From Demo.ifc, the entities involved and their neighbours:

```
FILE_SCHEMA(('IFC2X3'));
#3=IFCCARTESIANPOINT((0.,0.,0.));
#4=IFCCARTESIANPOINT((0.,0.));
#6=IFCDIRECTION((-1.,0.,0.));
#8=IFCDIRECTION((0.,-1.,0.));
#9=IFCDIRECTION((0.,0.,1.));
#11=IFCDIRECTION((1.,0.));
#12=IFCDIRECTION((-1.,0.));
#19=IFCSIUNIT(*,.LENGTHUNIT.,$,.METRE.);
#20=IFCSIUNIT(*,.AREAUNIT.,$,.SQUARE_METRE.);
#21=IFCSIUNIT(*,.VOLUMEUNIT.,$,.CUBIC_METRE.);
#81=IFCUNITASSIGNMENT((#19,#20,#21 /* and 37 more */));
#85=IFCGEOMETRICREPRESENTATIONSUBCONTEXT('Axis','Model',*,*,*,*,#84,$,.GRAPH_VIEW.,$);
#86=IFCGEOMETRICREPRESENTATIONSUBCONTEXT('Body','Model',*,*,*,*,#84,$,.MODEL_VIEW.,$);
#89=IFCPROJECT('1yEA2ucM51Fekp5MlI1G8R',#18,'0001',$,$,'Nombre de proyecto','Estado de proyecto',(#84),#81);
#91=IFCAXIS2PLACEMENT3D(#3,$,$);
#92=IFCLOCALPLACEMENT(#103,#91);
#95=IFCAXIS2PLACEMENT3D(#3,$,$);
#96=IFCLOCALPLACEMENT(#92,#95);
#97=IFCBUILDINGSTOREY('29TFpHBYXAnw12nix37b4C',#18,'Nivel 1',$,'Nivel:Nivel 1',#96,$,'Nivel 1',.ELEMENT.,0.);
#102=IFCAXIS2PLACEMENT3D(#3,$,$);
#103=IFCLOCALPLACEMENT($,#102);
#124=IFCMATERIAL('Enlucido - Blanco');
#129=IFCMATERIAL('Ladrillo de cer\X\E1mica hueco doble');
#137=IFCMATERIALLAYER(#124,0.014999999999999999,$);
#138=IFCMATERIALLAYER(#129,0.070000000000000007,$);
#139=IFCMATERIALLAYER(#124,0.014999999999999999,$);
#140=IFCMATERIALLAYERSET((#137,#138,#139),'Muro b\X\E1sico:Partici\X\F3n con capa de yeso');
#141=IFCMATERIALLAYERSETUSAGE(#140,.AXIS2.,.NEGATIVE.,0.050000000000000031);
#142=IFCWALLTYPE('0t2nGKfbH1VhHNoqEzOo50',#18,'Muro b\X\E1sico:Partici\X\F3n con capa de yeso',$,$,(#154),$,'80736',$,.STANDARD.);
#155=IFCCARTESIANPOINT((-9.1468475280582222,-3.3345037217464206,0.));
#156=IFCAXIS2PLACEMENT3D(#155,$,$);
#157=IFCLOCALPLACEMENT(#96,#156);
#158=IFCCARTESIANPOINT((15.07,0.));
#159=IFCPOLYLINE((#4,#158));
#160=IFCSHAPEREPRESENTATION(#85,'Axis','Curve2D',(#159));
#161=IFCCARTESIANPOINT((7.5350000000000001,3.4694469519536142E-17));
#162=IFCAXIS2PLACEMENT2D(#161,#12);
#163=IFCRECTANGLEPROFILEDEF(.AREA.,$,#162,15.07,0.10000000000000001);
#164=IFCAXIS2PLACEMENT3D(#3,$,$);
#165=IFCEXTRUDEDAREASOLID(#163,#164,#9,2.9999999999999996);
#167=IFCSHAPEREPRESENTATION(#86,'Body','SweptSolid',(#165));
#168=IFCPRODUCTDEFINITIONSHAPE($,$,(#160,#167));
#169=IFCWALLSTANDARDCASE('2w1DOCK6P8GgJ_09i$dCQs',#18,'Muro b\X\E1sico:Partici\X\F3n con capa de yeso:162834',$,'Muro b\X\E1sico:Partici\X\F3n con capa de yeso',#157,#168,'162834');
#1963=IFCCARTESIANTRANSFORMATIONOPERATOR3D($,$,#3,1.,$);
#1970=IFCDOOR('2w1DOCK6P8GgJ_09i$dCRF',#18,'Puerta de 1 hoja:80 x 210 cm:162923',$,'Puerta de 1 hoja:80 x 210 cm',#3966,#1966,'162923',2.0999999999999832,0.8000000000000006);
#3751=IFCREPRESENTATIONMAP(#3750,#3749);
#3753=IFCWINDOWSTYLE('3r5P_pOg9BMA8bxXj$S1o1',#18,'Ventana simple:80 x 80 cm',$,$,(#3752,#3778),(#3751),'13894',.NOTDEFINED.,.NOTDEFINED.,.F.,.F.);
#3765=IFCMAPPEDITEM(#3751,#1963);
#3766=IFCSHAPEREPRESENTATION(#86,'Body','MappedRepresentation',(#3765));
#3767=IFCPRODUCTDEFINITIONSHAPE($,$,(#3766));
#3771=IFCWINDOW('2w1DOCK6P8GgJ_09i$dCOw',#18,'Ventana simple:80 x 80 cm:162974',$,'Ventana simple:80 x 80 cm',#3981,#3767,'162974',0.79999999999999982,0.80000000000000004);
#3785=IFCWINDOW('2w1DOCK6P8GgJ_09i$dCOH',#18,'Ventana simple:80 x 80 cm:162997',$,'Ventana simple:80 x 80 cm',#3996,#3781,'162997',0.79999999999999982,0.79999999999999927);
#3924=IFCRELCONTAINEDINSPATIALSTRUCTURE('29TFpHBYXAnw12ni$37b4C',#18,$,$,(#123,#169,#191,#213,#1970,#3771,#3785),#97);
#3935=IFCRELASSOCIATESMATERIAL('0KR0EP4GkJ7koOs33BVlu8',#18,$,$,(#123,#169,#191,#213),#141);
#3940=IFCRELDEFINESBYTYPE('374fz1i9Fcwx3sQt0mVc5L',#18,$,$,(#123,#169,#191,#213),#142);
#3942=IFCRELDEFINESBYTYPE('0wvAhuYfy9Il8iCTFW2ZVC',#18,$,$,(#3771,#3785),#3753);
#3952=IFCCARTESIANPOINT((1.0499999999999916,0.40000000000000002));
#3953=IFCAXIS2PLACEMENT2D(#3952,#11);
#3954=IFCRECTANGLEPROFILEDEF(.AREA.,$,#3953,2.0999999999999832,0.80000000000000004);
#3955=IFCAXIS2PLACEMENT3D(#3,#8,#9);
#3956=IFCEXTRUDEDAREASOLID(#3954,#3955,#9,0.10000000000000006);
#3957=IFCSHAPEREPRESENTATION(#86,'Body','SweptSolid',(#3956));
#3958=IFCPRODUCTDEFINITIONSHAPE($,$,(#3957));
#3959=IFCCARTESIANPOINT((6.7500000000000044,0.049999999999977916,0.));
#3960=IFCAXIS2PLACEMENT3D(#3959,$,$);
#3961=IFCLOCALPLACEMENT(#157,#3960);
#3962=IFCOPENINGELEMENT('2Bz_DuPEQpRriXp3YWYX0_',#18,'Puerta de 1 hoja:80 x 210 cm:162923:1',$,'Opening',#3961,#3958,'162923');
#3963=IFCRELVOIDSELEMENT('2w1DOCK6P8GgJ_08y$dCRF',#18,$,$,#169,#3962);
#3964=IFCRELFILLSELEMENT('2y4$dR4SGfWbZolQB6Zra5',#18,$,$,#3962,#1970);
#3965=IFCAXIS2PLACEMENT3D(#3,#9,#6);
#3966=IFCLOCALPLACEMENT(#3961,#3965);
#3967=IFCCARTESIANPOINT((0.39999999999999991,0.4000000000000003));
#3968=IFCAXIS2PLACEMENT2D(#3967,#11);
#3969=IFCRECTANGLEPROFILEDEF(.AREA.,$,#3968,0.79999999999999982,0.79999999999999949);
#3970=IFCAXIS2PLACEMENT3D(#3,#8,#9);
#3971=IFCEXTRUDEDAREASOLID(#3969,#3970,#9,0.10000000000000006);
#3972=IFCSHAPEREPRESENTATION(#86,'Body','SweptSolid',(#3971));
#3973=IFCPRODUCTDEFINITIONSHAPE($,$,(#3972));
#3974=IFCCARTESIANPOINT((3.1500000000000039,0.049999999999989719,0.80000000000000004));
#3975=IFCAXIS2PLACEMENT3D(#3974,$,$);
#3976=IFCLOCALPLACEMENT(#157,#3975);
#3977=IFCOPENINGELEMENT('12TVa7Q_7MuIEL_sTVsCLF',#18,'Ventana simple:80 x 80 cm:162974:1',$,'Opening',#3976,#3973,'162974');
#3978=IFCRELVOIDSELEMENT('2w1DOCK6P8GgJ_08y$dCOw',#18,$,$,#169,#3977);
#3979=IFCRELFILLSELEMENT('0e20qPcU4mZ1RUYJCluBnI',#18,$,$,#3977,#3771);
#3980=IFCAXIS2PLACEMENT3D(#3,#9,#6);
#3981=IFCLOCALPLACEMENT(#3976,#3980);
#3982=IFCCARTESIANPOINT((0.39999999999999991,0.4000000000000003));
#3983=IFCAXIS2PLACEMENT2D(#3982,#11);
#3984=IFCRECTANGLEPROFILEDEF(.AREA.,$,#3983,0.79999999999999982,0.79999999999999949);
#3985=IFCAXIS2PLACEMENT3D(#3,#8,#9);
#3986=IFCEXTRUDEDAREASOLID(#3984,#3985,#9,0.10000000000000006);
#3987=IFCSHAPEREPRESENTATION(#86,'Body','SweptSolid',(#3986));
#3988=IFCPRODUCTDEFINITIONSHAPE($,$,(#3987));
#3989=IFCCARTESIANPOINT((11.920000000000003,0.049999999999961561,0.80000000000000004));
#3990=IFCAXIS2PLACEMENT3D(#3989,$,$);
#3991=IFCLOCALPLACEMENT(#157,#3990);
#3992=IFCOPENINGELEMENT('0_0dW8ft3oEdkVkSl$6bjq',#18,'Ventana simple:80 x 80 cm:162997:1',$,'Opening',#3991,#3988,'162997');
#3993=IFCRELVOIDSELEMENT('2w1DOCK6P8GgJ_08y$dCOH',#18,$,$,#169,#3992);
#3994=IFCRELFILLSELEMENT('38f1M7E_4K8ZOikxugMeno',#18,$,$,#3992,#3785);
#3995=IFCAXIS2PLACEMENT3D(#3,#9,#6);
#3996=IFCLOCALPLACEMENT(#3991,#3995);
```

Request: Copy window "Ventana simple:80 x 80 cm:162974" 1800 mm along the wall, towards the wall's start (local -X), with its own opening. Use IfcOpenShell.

```python
import ifcopenshell
import ifcopenshell.api.feature
import ifcopenshell.api.geometry
import ifcopenshell.api.root
import ifcopenshell.geom
import ifcopenshell.util.element
import ifcopenshell.util.placement
import ifcopenshell.util.shape
import ifcopenshell.util.unit

model = ifcopenshell.open("Demo.ifc")
unit_scale = ifcopenshell.util.unit.calculate_unit_scale(model)
settings = ifcopenshell.geom.settings()


def volume(element):
    """Net volume in cubic metres, openings subtracted."""
    shape = ifcopenshell.geom.create_shape(settings, element)
    return ifcopenshell.util.shape.get_volume(shape.geometry)


def reuse_history(source, copy):
    """copy_class also copies each property set's owner history, people and application; keep the originals."""
    for rel in copy.IsDefinedBy:
        if rel.is_a("IfcRelDefinesByProperties") and (history := rel.RelatingPropertyDefinition.OwnerHistory):
            rel.RelatingPropertyDefinition.OwnerHistory = source.OwnerHistory
            ifcopenshell.util.element.remove_deep2(model, history)


window = model.by_id(3771)
opening = window.FillsVoids[0].RelatingOpeningElement
wall = opening.VoidsElements[0].RelatingBuildingElement
before = volume(wall)
shift = ifcopenshell.util.placement.get_local_placement(wall.ObjectPlacement)[:3, 0] * -1.8 / unit_scale

# copy_class copies the void relationship, type, container and properties, but no geometry.
new_opening = ifcopenshell.api.root.copy_class(model, product=opening)
new_opening.Representation = ifcopenshell.util.element.copy_deep(
    model, opening.Representation, exclude=["IfcGeometricRepresentationContext", "IfcRepresentationMap"]
)
new_opening.Name = "Ventana simple:80 x 80 cm"
new_opening.Tag = None
new_window = ifcopenshell.api.root.copy_class(model, product=window)
new_window.Representation = ifcopenshell.util.element.copy_deep(
    model, window.Representation, exclude=["IfcGeometricRepresentationContext", "IfcRepresentationMap"]
)
new_window.Name = "Ventana simple:80 x 80 cm"
new_window.Tag = None
reuse_history(window, new_window)
fills = ifcopenshell.api.feature.add_filling(model, opening=new_opening, element=new_window)
fills.OwnerHistory = new_window.OwnerHistory  # required in IFC2X3

for old, new in ((opening, new_opening), (window, new_window)):
    matrix = ifcopenshell.util.placement.get_local_placement(old.ObjectPlacement)
    matrix[:3, 3] += shift
    ifcopenshell.api.geometry.edit_object_placement(model, product=new, matrix=matrix, is_si=False)

after = volume(wall)

print(f"wall volume {before:.3f} -> {after:.3f} m3")

model.write("Demo_updated.ifc")
```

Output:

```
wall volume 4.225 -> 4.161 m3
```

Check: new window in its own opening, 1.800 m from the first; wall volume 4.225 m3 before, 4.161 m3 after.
